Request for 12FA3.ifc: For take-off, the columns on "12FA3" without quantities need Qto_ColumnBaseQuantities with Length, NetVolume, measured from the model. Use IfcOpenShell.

First a look at what the model holds.

```python
import ifcopenshell
import ifcopenshell.util.element
import ifcopenshell.util.unit

model = ifcopenshell.open("12FA3.ifc")
print(model.schema)
for unit_type in ("LENGTHUNIT", "AREAUNIT", "VOLUMEUNIT"):
    print(unit_type, ifcopenshell.util.unit.calculate_unit_scale(model, unit_type))
storey = next(s for s in model.by_type("IfcBuildingStorey") if s.Name == "12FA3")
columns = [e for e in ifcopenshell.util.element.get_decomposition(storey) if e.is_a("IfcColumn")]
for e in sorted(columns, key=lambda e: e.id()):
    print(e.id(), e.is_a(), e.Name, list(ifcopenshell.util.element.get_psets(e, qtos_only=True)), sep=" | ")
```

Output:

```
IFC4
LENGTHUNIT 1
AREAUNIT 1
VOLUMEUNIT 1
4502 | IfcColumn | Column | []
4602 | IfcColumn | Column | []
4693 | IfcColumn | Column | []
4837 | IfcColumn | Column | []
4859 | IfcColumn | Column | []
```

```python
import ifcopenshell
import ifcopenshell.api.pset
import ifcopenshell.geom
import ifcopenshell.util.element
import ifcopenshell.util.shape
import ifcopenshell.util.unit

model = ifcopenshell.open("12FA3.ifc")
unit_scale = ifcopenshell.util.unit.calculate_unit_scale(model)
volume_scale = ifcopenshell.util.unit.calculate_unit_scale(model, "VOLUMEUNIT")
settings = ifcopenshell.geom.settings()

storey = next(s for s in model.by_type("IfcBuildingStorey") if s.Name == "12FA3")
columns = [e for e in ifcopenshell.util.element.get_decomposition(storey) if e.is_a("IfcColumn")]

for e in sorted(columns, key=lambda e: e.id()):
    if ifcopenshell.util.element.get_psets(e, qtos_only=True, should_inherit=False):
        continue
    # Geometry comes back in metres, in the element's own axes.
    shape = ifcopenshell.geom.create_shape(settings, e)
    values = {
        "Length": ifcopenshell.util.shape.get_z(shape.geometry) / unit_scale,
        "NetVolume": ifcopenshell.util.shape.get_volume(shape.geometry) / volume_scale,
    }
    qto = ifcopenshell.api.pset.add_qto(model, product=e, name="Qto_ColumnBaseQuantities")
    ifcopenshell.api.pset.edit_qto(model, qto=qto, properties=values)
    print(e.id(), {k: round(v, 3) for k, v in values.items()})

model.write("12FA3_rev.ifc")
```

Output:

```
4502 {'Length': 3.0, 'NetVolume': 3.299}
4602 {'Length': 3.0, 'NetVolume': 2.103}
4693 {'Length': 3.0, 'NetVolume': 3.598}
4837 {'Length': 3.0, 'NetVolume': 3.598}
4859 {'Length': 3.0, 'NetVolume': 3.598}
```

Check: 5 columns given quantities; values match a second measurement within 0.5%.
